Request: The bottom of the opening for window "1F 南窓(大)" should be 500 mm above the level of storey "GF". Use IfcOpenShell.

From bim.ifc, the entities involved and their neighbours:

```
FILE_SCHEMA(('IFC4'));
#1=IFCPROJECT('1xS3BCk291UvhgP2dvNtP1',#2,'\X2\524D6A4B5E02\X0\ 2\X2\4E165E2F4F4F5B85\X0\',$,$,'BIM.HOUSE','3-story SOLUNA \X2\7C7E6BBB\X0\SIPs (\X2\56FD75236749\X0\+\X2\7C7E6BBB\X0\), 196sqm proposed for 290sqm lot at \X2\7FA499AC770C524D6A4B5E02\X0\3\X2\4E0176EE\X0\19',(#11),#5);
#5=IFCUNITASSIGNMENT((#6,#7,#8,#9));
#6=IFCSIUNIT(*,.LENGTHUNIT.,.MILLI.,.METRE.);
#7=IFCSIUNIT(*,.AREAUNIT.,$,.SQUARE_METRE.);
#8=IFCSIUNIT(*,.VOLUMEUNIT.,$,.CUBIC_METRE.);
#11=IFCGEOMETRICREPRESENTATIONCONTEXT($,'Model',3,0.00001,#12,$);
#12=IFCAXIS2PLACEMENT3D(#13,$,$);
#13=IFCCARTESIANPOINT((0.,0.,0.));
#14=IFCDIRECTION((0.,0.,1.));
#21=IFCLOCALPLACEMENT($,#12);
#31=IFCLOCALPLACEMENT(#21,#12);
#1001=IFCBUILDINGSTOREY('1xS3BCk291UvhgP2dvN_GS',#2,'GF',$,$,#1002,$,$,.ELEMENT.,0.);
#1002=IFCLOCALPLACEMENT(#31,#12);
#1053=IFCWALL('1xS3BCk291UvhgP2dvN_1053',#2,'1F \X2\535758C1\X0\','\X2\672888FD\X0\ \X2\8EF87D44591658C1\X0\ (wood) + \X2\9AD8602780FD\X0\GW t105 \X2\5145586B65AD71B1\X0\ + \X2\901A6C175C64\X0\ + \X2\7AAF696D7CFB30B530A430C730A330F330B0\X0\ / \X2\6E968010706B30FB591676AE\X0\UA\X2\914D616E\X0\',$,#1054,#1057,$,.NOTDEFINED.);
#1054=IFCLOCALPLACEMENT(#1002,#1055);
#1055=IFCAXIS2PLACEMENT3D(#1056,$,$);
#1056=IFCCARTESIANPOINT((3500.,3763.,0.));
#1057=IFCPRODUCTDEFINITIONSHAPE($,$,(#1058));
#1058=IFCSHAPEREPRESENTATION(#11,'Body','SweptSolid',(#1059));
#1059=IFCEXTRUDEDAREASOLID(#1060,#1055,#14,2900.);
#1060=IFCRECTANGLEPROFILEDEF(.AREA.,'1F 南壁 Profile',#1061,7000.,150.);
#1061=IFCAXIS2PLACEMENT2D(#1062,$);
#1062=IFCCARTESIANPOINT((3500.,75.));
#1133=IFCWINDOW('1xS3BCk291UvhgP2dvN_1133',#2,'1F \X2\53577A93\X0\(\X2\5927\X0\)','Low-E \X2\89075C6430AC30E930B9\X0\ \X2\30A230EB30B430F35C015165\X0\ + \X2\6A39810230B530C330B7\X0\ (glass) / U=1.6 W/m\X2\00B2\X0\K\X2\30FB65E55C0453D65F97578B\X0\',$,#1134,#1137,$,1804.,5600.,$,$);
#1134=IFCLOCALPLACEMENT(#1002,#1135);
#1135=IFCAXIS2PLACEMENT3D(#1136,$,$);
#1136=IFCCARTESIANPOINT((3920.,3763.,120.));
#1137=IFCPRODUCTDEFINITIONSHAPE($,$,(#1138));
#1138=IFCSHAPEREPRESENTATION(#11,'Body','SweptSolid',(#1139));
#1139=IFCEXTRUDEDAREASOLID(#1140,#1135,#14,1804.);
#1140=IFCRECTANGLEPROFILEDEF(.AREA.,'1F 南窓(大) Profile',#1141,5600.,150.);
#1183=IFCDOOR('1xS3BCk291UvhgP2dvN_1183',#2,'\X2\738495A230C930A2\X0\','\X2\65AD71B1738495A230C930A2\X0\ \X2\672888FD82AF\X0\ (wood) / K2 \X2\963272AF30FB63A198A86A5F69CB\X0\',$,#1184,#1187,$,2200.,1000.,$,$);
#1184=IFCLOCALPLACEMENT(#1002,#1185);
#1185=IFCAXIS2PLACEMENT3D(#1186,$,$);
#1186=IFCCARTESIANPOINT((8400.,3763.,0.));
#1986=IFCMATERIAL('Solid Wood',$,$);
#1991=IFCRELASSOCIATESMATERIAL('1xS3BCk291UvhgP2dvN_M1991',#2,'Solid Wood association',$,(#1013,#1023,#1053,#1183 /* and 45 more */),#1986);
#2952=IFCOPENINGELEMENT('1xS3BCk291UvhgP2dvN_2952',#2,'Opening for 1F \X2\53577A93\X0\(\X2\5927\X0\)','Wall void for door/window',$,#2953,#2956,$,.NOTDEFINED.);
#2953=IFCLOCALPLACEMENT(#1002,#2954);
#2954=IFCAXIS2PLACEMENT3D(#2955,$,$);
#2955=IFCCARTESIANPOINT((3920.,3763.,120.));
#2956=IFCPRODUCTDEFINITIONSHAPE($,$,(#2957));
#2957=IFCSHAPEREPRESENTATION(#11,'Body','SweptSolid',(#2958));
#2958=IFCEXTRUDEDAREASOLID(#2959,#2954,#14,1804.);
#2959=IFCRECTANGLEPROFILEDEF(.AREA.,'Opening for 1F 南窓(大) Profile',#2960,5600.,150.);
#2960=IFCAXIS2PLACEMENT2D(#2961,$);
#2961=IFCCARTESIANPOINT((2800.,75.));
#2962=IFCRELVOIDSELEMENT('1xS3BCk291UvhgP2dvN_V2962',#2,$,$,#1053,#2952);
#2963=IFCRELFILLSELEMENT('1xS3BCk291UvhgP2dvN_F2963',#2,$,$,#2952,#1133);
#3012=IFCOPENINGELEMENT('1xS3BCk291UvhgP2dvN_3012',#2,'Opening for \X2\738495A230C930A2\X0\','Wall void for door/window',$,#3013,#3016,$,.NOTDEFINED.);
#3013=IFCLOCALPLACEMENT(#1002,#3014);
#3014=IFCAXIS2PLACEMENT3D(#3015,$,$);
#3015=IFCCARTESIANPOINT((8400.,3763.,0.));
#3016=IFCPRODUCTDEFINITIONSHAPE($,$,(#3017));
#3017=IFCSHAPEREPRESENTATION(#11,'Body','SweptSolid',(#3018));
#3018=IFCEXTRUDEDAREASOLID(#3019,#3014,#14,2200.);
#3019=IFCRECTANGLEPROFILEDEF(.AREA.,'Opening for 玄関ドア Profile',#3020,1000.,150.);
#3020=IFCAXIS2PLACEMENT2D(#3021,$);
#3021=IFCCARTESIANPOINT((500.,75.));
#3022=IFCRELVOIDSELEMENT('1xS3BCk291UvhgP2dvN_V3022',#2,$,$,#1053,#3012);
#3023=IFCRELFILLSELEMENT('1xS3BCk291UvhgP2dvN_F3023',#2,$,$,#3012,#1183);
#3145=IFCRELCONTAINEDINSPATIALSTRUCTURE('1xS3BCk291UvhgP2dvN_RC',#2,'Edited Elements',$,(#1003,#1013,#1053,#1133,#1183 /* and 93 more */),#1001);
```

```python
import numpy as np
import ifcopenshell
import ifcopenshell.api.geometry
import ifcopenshell.geom
import ifcopenshell.util.element
import ifcopenshell.util.placement
import ifcopenshell.util.shape
import ifcopenshell.util.unit

model = ifcopenshell.open("bim.ifc")
unit_scale = ifcopenshell.util.unit.calculate_unit_scale(model)

window = model.by_id(1133)
opening = window.FillsVoids[0].RelatingOpeningElement
storey = ifcopenshell.util.element.get_container(window, ifc_class="IfcBuildingStorey")
level = ifcopenshell.util.placement.get_local_placement(storey.ObjectPlacement)[2, 3]

# The opening's origin need not be at the sill, so measure its lowest point.
shape = ifcopenshell.geom.create_shape(ifcopenshell.geom.settings(), opening)
bottom = ifcopenshell.util.shape.get_shape_bottom_elevation(shape, shape.geometry) / unit_scale
dz = level + 500.0 - bottom

shift = np.array([0.0, 0.0, dz])
# The window is not placed relative to its opening, so move both.
for product in (opening, window):
    matrix = ifcopenshell.util.placement.get_local_placement(product.ObjectPlacement)
    matrix[:3, 3] += shift
    ifcopenshell.api.geometry.edit_object_placement(model, product=product, matrix=matrix, is_si=False)

print(f"moved by {dz * unit_scale:+.3f} m")

model.write("bim_updated.ifc")
```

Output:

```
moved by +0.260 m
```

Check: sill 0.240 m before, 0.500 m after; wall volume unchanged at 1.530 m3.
